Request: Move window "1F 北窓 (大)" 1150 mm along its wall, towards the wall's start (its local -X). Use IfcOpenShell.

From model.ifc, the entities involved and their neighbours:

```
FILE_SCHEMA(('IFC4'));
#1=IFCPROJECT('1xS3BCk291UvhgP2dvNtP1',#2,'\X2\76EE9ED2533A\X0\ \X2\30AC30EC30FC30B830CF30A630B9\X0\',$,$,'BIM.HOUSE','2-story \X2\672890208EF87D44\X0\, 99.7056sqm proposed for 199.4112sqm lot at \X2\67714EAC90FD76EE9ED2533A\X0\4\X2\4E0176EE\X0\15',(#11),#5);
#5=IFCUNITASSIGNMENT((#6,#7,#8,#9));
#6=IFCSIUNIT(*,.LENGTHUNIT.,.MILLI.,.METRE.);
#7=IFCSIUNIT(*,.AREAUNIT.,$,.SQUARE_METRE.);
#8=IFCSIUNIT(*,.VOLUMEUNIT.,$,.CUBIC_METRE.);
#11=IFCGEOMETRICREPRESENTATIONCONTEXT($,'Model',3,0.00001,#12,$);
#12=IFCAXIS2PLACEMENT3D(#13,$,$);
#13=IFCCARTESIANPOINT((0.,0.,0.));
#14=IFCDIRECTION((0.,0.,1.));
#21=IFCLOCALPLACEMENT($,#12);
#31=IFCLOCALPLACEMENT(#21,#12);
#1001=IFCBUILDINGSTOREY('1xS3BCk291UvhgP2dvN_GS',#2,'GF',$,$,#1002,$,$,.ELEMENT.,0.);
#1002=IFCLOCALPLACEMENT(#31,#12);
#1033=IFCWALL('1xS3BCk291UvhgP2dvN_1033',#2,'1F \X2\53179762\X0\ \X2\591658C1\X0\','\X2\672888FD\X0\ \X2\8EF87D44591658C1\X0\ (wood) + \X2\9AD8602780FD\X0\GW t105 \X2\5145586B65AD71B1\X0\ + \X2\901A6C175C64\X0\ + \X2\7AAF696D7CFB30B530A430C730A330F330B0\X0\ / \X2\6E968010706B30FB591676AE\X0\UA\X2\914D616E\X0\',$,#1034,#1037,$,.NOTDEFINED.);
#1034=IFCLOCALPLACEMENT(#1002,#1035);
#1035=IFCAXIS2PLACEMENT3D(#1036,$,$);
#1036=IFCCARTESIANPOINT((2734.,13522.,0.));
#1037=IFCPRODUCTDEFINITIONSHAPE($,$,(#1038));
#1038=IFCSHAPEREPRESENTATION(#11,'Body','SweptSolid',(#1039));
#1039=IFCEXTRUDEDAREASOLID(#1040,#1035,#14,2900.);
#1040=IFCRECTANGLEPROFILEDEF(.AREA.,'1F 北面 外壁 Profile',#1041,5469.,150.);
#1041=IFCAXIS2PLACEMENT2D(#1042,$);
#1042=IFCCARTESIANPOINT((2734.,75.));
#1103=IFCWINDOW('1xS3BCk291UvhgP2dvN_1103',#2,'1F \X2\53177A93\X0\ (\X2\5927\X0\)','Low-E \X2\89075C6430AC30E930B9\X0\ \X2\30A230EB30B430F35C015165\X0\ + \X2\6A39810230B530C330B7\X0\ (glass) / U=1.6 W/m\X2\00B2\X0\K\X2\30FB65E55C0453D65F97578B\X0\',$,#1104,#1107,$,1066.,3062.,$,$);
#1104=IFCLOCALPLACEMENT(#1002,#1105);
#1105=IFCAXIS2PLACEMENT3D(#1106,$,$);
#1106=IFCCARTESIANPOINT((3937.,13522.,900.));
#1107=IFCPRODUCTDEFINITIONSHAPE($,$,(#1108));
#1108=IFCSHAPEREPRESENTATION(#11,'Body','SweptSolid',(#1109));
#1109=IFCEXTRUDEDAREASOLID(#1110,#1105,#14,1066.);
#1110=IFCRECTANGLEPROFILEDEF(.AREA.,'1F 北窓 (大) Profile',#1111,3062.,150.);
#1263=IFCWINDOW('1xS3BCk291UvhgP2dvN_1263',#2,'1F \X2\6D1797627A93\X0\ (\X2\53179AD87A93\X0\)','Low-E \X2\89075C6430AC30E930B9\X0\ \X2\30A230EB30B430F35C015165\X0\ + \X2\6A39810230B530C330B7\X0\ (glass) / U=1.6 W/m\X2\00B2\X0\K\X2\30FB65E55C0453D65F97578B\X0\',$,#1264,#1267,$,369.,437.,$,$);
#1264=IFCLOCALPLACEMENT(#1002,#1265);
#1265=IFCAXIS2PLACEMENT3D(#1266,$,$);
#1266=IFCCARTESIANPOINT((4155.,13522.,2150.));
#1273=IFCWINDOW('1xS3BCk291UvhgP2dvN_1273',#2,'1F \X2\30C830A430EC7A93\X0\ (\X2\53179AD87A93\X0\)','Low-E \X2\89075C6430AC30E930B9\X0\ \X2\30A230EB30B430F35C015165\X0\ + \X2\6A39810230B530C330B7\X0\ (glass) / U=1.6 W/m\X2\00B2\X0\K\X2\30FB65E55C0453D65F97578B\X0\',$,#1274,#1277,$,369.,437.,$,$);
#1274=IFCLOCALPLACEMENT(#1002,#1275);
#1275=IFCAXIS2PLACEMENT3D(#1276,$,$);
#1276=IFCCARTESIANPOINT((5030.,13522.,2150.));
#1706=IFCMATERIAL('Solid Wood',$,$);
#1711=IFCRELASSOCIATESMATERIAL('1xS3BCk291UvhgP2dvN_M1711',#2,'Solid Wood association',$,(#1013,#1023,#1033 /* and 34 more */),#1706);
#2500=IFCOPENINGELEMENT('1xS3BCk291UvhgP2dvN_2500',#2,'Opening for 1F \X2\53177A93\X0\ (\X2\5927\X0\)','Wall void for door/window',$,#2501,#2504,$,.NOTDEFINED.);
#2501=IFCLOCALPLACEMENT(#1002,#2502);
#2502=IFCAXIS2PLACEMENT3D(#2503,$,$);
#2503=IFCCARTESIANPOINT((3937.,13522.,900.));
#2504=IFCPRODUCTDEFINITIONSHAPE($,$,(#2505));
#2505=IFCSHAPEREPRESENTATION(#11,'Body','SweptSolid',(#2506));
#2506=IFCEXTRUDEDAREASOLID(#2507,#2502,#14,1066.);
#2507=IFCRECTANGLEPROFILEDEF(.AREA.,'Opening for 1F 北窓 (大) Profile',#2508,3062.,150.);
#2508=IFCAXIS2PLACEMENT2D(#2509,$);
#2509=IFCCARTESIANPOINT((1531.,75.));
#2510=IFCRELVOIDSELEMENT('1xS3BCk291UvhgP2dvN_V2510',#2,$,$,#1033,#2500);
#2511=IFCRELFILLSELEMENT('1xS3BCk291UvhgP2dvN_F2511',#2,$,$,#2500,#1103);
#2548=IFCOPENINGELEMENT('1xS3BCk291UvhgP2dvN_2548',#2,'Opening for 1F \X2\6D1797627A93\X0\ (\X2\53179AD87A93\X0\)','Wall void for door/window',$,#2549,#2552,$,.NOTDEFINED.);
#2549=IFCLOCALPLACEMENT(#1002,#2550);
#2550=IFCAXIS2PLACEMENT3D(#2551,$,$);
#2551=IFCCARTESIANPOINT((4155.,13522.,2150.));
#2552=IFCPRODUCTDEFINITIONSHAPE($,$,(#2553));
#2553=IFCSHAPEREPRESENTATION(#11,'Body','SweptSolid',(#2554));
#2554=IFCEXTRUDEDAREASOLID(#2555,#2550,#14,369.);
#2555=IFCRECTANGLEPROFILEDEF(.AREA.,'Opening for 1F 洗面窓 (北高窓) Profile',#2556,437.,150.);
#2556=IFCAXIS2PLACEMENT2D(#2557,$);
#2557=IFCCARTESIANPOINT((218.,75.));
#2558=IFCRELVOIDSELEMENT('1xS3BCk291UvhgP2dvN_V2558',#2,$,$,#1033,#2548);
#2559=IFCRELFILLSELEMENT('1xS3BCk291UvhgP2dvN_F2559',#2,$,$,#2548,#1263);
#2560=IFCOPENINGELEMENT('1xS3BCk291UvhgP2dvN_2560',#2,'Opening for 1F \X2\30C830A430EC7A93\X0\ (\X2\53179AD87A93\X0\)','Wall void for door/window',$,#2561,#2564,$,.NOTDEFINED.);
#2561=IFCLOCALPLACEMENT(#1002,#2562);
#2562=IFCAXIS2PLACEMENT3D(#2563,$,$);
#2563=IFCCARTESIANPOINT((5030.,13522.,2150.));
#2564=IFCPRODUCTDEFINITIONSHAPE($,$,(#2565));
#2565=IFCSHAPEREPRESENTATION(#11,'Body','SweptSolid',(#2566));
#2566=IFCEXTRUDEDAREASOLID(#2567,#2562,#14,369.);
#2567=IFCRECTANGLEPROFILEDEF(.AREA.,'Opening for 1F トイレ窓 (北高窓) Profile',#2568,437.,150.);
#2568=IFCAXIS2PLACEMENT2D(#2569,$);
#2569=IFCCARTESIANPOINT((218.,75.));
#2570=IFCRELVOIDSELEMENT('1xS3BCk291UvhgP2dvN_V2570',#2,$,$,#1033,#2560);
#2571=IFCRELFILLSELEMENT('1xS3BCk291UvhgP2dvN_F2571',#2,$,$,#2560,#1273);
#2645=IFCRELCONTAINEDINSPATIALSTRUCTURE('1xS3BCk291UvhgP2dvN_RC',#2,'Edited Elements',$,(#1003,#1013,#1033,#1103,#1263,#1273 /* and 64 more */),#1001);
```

```python
import ifcopenshell
import ifcopenshell.api.geometry
import ifcopenshell.util.placement
import ifcopenshell.util.unit

model = ifcopenshell.open("model.ifc")
unit_scale = ifcopenshell.util.unit.calculate_unit_scale(model)

window = model.by_guid("1xS3BCk291UvhgP2dvN_1103")
opening = window.FillsVoids[0].RelatingOpeningElement
wall = opening.VoidsElements[0].RelatingBuildingElement

wall_matrix = ifcopenshell.util.placement.get_local_placement(wall.ObjectPlacement)
shift = wall_matrix[:3, 0] * -1.15 / unit_scale
before = ifcopenshell.util.placement.get_local_placement(window.ObjectPlacement)[:3, 3].copy()

# The window is not placed relative to its opening, so move both.
for product in (opening, window):
    matrix = ifcopenshell.util.placement.get_local_placement(product.ObjectPlacement)
    matrix[:3, 3] += shift
    ifcopenshell.api.geometry.edit_object_placement(model, product=product, matrix=matrix, is_si=False)

after = ifcopenshell.util.placement.get_local_placement(window.ObjectPlacement)[:3, 3]
print("window moved by", (after - before).round(3) + 0.0)

model.write("model_rev.ifc")
```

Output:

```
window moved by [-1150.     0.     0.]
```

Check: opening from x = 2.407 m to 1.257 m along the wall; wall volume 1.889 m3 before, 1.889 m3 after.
